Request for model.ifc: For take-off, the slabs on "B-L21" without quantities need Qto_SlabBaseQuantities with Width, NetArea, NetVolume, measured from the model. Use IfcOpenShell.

First a look at what the model holds.

```python
import ifcopenshell
import ifcopenshell.util.element
import ifcopenshell.util.unit

model = ifcopenshell.open("model.ifc")
print(model.schema)
for unit_type in ("LENGTHUNIT", "AREAUNIT", "VOLUMEUNIT"):
    print(unit_type, ifcopenshell.util.unit.calculate_unit_scale(model, unit_type))
storey = next(s for s in model.by_type("IfcBuildingStorey") if s.Name == "B-L21")
slabs = [e for e in ifcopenshell.util.element.get_decomposition(storey) if e.is_a("IfcSlab")]
for e in sorted(slabs, key=lambda e: e.id()):
    print(e.id(), e.is_a(), e.Name, list(ifcopenshell.util.element.get_psets(e, qtos_only=True)), sep=" | ")
```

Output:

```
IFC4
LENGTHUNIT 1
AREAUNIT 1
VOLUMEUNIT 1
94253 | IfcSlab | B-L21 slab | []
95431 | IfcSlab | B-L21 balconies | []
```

```python
import ifcopenshell
import ifcopenshell.api.pset
import ifcopenshell.geom
import ifcopenshell.util.element
import ifcopenshell.util.shape
import ifcopenshell.util.unit

model = ifcopenshell.open("model.ifc")
unit_scale = ifcopenshell.util.unit.calculate_unit_scale(model)
area_scale = ifcopenshell.util.unit.calculate_unit_scale(model, "AREAUNIT")
volume_scale = ifcopenshell.util.unit.calculate_unit_scale(model, "VOLUMEUNIT")
settings = ifcopenshell.geom.settings()

storey = next(s for s in model.by_type("IfcBuildingStorey") if s.Name == "B-L21")
slabs = [e for e in ifcopenshell.util.element.get_decomposition(storey) if e.is_a("IfcSlab")]

for e in sorted(slabs, key=lambda e: e.id()):
    if ifcopenshell.util.element.get_psets(e, qtos_only=True, should_inherit=False):
        continue
    # Geometry comes back in metres, in the element's own axes.
    shape = ifcopenshell.geom.create_shape(settings, e)
    values = {
        "Width": ifcopenshell.util.shape.get_z(shape.geometry) / unit_scale,
        "NetArea": ifcopenshell.util.shape.get_footprint_area(shape.geometry) / area_scale,
        "NetVolume": ifcopenshell.util.shape.get_volume(shape.geometry) / volume_scale,
    }
    qto = ifcopenshell.api.pset.add_qto(model, product=e, name="Qto_SlabBaseQuantities")
    ifcopenshell.api.pset.edit_qto(model, qto=qto, properties=values)
    print(e.id(), {k: round(v, 3) for k, v in values.items()})

model.write("model_v2.ifc")
```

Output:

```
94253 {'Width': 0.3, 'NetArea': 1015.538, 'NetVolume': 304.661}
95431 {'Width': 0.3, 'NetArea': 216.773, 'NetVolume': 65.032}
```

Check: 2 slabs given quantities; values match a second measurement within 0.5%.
